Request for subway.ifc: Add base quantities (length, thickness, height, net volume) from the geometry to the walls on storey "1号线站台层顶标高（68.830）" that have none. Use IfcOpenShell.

First a look at what the model holds.

```python
import ifcopenshell
import ifcopenshell.util.element
import ifcopenshell.util.unit

model = ifcopenshell.open("subway.ifc")
print(model.schema)
for unit_type in ("LENGTHUNIT", "AREAUNIT", "VOLUMEUNIT"):
    print(unit_type, ifcopenshell.util.unit.calculate_unit_scale(model, unit_type))
storey = next(s for s in model.by_type("IfcBuildingStorey") if s.Name == "1号线站台层顶标高（68.830）")
walls = [e for e in ifcopenshell.util.element.get_decomposition(storey) if e.is_a("IfcWall")]
for e in sorted(walls, key=lambda e: e.id()):
    print(e.id(), e.is_a(), e.Name, list(ifcopenshell.util.element.get_psets(e, qtos_only=True)), sep=" | ")
```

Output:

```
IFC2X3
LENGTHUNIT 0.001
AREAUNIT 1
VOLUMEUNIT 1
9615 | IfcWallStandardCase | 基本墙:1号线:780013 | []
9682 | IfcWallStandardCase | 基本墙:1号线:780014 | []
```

```python
import ifcopenshell
import ifcopenshell.api.pset
import ifcopenshell.geom
import ifcopenshell.util.element
import ifcopenshell.util.shape
import ifcopenshell.util.unit

model = ifcopenshell.open("subway.ifc")
unit_scale = ifcopenshell.util.unit.calculate_unit_scale(model)
volume_scale = ifcopenshell.util.unit.calculate_unit_scale(model, "VOLUMEUNIT")
settings = ifcopenshell.geom.settings()

storey = next(s for s in model.by_type("IfcBuildingStorey") if s.Name == "1号线站台层顶标高（68.830）")
walls = [e for e in ifcopenshell.util.element.get_decomposition(storey) if e.is_a("IfcWall")]

for e in sorted(walls, key=lambda e: e.id()):
    if ifcopenshell.util.element.get_psets(e, qtos_only=True, should_inherit=False):
        continue
    # Geometry comes back in metres, in the element's own axes.
    shape = ifcopenshell.geom.create_shape(settings, e)
    values = {
        "Length": ifcopenshell.util.shape.get_x(shape.geometry) / unit_scale,
        "Width": ifcopenshell.util.shape.get_y(shape.geometry) / unit_scale,
        "Height": ifcopenshell.util.shape.get_z(shape.geometry) / unit_scale,
        "NetVolume": ifcopenshell.util.shape.get_volume(shape.geometry) / volume_scale,
    }
    qto = ifcopenshell.api.pset.add_qto(model, product=e, name="BaseQuantities")
    ifcopenshell.api.pset.edit_qto(model, qto=qto, properties=values)
    print(e.id(), {k: round(v, 3) for k, v in values.items()})

model.write("subway_rev.ifc")
```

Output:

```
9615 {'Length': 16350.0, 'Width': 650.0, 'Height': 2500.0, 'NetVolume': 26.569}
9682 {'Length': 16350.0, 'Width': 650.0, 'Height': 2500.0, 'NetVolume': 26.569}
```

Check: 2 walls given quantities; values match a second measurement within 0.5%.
